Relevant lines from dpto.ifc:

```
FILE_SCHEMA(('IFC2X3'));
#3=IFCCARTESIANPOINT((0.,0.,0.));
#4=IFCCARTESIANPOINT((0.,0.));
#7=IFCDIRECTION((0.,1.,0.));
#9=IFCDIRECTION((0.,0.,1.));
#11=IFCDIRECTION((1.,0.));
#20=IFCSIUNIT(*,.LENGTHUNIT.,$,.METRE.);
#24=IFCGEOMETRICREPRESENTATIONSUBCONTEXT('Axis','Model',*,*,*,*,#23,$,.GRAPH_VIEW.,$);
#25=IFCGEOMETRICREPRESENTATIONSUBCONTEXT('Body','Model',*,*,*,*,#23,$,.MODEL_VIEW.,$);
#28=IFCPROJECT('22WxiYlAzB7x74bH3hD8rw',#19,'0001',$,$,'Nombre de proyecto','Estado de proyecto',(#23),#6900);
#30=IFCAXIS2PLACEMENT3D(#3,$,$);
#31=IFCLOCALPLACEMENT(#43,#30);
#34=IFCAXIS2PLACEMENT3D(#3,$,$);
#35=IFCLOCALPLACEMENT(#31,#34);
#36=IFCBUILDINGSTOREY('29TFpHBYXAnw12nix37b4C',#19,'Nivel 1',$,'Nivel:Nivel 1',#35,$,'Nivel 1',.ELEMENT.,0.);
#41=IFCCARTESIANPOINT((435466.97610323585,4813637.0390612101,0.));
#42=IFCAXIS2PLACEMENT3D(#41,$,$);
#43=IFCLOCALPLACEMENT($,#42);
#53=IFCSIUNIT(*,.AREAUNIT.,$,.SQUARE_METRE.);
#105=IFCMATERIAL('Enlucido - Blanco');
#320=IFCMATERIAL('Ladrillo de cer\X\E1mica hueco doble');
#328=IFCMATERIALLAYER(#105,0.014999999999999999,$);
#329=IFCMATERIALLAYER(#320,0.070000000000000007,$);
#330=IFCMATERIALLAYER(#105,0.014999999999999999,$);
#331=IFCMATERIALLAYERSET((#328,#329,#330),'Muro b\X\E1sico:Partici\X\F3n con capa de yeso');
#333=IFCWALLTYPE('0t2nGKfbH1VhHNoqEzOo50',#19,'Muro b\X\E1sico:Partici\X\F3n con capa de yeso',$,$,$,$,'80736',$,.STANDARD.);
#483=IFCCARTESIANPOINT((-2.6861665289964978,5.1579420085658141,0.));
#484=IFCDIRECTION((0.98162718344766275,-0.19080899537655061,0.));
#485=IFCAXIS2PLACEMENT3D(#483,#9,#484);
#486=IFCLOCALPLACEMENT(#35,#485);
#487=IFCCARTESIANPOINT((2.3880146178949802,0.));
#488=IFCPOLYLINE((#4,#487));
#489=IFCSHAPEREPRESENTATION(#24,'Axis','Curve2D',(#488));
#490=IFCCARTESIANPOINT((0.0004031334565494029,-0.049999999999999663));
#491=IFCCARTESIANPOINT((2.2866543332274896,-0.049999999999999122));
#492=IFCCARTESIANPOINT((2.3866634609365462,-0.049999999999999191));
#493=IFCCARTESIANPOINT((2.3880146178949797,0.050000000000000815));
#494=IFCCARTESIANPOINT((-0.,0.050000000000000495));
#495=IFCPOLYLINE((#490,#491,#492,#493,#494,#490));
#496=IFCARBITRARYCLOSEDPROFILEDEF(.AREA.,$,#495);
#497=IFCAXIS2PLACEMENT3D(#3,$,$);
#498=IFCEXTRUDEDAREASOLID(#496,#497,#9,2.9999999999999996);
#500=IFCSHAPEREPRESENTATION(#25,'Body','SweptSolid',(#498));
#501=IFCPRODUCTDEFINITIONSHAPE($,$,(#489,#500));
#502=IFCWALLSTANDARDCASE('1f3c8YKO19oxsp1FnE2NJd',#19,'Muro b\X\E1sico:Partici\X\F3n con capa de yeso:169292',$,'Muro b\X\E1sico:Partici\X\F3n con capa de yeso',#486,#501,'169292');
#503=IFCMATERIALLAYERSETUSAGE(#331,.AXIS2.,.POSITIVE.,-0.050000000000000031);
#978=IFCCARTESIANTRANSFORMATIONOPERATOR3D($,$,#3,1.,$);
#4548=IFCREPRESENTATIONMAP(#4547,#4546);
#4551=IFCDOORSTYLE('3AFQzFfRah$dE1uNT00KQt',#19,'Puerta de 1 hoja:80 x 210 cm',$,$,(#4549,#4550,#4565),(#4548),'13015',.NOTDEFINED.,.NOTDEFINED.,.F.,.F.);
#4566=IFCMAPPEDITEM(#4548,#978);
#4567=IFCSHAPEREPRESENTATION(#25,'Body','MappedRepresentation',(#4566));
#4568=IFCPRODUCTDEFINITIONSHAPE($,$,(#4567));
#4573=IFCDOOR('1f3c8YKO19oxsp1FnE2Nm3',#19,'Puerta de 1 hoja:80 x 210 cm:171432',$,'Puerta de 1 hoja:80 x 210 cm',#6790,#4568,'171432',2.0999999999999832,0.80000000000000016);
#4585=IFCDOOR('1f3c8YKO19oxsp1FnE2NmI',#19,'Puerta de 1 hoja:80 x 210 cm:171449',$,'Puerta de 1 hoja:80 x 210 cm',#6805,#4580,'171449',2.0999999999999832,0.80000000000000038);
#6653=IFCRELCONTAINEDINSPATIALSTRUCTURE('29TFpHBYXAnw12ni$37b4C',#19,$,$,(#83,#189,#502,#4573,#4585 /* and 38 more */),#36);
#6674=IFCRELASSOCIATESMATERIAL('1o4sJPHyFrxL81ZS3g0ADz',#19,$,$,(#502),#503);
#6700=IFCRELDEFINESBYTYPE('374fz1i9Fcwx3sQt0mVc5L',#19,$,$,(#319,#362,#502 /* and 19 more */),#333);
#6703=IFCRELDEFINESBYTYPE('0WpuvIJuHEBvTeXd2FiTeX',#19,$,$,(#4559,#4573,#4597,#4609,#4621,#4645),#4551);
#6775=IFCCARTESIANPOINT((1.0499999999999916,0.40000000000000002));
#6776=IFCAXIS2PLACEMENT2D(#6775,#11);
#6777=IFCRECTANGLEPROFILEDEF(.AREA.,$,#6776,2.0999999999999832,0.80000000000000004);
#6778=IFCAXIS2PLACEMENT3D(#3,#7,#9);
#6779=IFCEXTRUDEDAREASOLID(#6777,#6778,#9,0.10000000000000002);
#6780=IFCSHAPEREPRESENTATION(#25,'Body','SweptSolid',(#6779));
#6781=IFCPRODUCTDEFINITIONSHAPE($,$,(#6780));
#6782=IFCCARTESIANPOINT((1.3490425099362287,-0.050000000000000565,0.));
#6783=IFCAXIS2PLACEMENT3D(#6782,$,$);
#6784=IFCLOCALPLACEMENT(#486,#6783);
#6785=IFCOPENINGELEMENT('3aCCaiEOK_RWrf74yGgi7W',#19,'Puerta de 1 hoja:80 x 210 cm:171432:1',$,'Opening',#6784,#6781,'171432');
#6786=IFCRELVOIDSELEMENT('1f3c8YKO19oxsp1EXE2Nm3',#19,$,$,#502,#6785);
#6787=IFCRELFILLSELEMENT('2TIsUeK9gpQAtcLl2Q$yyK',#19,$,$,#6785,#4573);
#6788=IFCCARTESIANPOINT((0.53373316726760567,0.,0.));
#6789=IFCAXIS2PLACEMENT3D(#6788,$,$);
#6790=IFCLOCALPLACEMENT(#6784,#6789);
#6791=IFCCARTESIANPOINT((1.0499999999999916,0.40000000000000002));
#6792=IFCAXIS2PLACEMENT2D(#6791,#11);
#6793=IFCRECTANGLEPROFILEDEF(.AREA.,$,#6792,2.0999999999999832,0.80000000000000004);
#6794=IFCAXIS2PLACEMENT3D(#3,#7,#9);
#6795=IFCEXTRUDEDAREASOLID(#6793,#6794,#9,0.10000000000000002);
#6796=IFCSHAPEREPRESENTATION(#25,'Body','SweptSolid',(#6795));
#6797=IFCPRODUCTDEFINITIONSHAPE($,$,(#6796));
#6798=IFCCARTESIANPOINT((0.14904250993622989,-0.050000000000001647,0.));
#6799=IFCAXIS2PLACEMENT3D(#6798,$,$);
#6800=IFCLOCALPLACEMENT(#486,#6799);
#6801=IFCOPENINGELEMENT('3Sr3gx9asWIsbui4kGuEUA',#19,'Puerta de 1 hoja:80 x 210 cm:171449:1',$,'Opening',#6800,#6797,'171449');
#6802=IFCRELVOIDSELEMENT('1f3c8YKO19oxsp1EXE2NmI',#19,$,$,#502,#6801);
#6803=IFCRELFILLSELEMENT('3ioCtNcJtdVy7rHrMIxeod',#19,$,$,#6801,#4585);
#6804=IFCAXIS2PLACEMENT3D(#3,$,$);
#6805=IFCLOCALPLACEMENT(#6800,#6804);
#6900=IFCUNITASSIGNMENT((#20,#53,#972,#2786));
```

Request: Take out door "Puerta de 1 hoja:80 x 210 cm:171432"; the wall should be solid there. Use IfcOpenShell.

```python
import ifcopenshell
import ifcopenshell.api.feature
import ifcopenshell.api.root
import ifcopenshell.geom
import ifcopenshell.util.shape

model = ifcopenshell.open("dpto.ifc")
settings = ifcopenshell.geom.settings()


def volume(element):
    """Net volume in cubic metres, openings subtracted."""
    shape = ifcopenshell.geom.create_shape(settings, element)
    return ifcopenshell.util.shape.get_volume(shape.geometry)


door = model.by_guid("1f3c8YKO19oxsp1FnE2Nm3")
opening = door.FillsVoids[0].RelatingOpeningElement
wall = opening.VoidsElements[0].RelatingBuildingElement
before = volume(wall)

ifcopenshell.api.root.remove_product(model, product=door)
ifcopenshell.api.feature.remove_feature(model, feature=opening)

after = volume(wall)

print(f"wall volume {before:.3f} -> {after:.3f} m3")

model.write("dpto_v2.ifc")
```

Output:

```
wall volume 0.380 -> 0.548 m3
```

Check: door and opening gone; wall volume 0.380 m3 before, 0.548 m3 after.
